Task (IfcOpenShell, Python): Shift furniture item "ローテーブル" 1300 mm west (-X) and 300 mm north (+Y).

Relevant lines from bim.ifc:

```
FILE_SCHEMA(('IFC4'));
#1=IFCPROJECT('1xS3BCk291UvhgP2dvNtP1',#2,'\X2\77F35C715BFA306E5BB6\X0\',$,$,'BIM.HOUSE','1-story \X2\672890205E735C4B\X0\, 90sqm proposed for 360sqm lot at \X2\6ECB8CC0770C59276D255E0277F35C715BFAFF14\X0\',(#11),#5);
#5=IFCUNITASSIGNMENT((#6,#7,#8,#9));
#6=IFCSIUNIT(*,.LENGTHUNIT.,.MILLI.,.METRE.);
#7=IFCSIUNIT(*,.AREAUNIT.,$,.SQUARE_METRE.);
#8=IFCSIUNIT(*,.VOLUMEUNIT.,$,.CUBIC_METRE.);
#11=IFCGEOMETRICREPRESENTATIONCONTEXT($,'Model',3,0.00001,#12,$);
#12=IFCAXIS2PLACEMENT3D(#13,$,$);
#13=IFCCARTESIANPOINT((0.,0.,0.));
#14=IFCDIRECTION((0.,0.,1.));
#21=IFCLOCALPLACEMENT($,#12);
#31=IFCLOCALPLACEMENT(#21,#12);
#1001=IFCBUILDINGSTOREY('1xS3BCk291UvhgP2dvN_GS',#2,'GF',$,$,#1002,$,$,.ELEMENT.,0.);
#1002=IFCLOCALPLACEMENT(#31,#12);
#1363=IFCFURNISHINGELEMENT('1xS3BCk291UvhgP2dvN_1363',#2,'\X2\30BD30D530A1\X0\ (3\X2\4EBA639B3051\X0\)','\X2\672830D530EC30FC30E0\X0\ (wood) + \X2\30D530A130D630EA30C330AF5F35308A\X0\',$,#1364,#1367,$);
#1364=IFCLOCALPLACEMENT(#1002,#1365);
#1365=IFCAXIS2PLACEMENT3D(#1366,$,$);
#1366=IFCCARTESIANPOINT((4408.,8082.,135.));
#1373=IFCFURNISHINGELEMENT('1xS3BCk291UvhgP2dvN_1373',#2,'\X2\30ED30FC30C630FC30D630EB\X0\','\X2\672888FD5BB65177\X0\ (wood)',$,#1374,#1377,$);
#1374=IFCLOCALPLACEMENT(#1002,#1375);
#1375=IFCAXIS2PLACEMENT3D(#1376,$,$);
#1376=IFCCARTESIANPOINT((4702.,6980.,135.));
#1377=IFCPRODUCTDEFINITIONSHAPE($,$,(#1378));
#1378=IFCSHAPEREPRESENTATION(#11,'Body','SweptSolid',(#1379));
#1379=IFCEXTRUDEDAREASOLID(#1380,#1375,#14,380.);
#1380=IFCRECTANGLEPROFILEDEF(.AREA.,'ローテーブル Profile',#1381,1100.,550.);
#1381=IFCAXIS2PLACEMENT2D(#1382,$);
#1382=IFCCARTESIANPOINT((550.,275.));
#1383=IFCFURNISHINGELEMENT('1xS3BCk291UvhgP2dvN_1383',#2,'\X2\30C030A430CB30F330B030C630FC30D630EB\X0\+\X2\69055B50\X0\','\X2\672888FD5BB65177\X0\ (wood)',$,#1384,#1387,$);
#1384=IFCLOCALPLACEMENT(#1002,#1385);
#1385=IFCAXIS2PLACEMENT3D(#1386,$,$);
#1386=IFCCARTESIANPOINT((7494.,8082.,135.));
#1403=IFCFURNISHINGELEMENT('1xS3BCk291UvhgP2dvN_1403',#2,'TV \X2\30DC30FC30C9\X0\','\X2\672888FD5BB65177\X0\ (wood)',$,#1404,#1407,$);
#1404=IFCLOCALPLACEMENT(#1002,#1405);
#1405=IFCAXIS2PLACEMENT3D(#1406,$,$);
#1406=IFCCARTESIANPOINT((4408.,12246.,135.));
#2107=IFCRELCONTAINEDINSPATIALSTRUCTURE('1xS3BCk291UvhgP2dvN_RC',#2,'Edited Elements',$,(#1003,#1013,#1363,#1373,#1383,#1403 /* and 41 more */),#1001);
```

```python
import ifcopenshell
import ifcopenshell.api.geometry
import ifcopenshell.util.placement
import ifcopenshell.util.unit

model = ifcopenshell.open("bim.ifc")
unit_scale = ifcopenshell.util.unit.calculate_unit_scale(model)

item = model.by_guid("1xS3BCk291UvhgP2dvN_1373")
matrix = ifcopenshell.util.placement.get_local_placement(item.ObjectPlacement)
matrix[0, 3] -= 1.3 / unit_scale
matrix[1, 3] += 0.3 / unit_scale
ifcopenshell.api.geometry.edit_object_placement(model, product=item, matrix=matrix, is_si=False)

print(ifcopenshell.util.placement.get_local_placement(item.ObjectPlacement).round(3) + 0.0)

model.write("bim-out.ifc")
```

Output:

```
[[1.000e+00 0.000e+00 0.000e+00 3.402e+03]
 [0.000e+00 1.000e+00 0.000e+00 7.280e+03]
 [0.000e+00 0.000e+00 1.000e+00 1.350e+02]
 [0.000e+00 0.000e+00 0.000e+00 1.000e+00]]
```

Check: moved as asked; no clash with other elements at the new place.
